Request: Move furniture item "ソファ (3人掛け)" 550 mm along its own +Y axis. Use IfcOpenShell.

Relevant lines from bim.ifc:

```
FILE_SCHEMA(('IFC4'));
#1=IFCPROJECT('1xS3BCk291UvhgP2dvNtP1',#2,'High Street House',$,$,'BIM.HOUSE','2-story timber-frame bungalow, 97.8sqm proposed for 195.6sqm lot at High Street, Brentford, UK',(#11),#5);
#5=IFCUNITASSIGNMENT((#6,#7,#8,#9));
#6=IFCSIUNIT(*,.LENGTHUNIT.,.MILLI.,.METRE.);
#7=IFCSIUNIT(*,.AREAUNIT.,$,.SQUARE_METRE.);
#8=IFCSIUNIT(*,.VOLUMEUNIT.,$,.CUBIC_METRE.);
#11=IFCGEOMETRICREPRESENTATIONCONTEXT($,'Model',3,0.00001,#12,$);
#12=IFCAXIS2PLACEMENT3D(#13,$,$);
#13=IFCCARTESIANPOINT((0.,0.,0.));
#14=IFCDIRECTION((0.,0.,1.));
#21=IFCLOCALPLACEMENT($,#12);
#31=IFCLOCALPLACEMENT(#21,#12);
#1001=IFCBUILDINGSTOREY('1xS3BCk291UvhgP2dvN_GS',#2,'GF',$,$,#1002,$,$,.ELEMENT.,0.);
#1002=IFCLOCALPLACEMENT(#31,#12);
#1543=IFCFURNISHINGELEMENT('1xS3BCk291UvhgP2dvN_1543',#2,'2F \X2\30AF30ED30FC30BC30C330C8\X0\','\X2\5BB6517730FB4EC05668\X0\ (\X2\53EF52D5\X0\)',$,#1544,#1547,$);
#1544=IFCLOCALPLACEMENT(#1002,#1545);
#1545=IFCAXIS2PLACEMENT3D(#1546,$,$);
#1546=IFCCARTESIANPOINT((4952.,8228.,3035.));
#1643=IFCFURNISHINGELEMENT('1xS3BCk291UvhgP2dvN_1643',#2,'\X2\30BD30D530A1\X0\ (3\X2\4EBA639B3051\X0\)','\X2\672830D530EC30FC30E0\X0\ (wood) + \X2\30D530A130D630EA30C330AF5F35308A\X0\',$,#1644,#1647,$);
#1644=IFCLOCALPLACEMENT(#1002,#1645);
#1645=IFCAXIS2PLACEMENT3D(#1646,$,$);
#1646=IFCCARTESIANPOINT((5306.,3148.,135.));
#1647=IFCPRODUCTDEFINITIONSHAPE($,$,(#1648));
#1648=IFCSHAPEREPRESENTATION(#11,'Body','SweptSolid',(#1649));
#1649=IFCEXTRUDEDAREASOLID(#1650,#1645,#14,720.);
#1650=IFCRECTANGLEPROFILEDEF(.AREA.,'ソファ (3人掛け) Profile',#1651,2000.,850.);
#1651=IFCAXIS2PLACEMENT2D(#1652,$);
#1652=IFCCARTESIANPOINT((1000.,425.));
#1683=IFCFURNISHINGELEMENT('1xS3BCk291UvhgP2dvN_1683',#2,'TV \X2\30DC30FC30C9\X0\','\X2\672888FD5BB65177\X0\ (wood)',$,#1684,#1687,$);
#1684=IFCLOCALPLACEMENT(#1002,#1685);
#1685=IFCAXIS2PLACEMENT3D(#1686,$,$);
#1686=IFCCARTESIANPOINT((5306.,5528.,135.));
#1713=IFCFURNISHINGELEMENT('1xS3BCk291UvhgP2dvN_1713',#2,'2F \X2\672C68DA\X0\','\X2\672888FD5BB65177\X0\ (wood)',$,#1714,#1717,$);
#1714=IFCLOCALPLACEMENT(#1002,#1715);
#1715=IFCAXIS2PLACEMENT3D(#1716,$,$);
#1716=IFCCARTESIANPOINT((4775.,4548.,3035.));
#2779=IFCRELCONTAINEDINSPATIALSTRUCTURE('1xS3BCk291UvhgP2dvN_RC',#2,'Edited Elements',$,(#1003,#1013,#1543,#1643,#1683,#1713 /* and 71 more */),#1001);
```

```python
import ifcopenshell
import ifcopenshell.api.geometry
import ifcopenshell.util.placement
import ifcopenshell.util.unit

model = ifcopenshell.open("bim.ifc")
unit_scale = ifcopenshell.util.unit.calculate_unit_scale(model)

item = model.by_id(1643)
matrix = ifcopenshell.util.placement.get_local_placement(item.ObjectPlacement)
matrix[:3, 3] += matrix[:3, 1] * 0.55 / unit_scale
ifcopenshell.api.geometry.edit_object_placement(model, product=item, matrix=matrix, is_si=False)

print(ifcopenshell.util.placement.get_local_placement(item.ObjectPlacement).round(3) + 0.0)

model.write("bim_rev.ifc")
```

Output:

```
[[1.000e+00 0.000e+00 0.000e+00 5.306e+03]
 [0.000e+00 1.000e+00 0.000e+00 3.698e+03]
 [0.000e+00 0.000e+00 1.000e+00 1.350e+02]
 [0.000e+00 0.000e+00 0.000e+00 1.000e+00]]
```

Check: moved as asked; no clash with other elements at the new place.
